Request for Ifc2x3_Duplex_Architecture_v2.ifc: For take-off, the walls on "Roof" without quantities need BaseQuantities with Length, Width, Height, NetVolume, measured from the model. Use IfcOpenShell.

First a look at what the model holds.

```python
import ifcopenshell
import ifcopenshell.util.element
import ifcopenshell.util.unit

model = ifcopenshell.open("Ifc2x3_Duplex_Architecture_v2.ifc")
print(model.schema)
for unit_type in ("LENGTHUNIT", "AREAUNIT", "VOLUMEUNIT"):
    print(unit_type, ifcopenshell.util.unit.calculate_unit_scale(model, unit_type))
storey = next(s for s in model.by_type("IfcBuildingStorey") if s.Name == "Roof")
walls = [e for e in ifcopenshell.util.element.get_decomposition(storey) if e.is_a("IfcWall")]
for e in sorted(walls, key=lambda e: e.id()):
    print(e.id(), e.is_a(), e.Name, list(ifcopenshell.util.element.get_psets(e, qtos_only=True)), sep=" | ")
```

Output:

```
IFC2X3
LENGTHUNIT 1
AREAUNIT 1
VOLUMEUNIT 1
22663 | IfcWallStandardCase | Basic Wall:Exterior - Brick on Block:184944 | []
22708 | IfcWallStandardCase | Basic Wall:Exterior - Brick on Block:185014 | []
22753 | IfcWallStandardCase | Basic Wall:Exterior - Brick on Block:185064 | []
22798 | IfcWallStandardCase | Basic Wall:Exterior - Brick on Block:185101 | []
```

```python
import ifcopenshell
import ifcopenshell.api.pset
import ifcopenshell.geom
import ifcopenshell.util.element
import ifcopenshell.util.shape
import ifcopenshell.util.unit

model = ifcopenshell.open("Ifc2x3_Duplex_Architecture_v2.ifc")
unit_scale = ifcopenshell.util.unit.calculate_unit_scale(model)
volume_scale = ifcopenshell.util.unit.calculate_unit_scale(model, "VOLUMEUNIT")
settings = ifcopenshell.geom.settings()

storey = next(s for s in model.by_type("IfcBuildingStorey") if s.Name == "Roof")
walls = [e for e in ifcopenshell.util.element.get_decomposition(storey) if e.is_a("IfcWall")]

for e in sorted(walls, key=lambda e: e.id()):
    if ifcopenshell.util.element.get_psets(e, qtos_only=True, should_inherit=False):
        continue
    # Geometry comes back in metres, in the element's own axes.
    shape = ifcopenshell.geom.create_shape(settings, e)
    values = {
        "Length": ifcopenshell.util.shape.get_x(shape.geometry) / unit_scale,
        "Width": ifcopenshell.util.shape.get_y(shape.geometry) / unit_scale,
        "Height": ifcopenshell.util.shape.get_z(shape.geometry) / unit_scale,
        "NetVolume": ifcopenshell.util.shape.get_volume(shape.geometry) / volume_scale,
    }
    qto = ifcopenshell.api.pset.add_qto(model, product=e, name="BaseQuantities")
    ifcopenshell.api.pset.edit_qto(model, qto=qto, properties=values)
    print(e.id(), {k: round(v, 3) for k, v in values.items()})

model.write("Ifc2x3_Duplex_Architecture_v2_edited.ifc")
```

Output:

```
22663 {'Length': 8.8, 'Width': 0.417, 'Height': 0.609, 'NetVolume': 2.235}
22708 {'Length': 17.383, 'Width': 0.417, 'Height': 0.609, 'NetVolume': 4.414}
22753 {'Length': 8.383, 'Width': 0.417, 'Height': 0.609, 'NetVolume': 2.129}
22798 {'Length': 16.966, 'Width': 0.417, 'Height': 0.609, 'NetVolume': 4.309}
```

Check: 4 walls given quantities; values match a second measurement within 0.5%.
